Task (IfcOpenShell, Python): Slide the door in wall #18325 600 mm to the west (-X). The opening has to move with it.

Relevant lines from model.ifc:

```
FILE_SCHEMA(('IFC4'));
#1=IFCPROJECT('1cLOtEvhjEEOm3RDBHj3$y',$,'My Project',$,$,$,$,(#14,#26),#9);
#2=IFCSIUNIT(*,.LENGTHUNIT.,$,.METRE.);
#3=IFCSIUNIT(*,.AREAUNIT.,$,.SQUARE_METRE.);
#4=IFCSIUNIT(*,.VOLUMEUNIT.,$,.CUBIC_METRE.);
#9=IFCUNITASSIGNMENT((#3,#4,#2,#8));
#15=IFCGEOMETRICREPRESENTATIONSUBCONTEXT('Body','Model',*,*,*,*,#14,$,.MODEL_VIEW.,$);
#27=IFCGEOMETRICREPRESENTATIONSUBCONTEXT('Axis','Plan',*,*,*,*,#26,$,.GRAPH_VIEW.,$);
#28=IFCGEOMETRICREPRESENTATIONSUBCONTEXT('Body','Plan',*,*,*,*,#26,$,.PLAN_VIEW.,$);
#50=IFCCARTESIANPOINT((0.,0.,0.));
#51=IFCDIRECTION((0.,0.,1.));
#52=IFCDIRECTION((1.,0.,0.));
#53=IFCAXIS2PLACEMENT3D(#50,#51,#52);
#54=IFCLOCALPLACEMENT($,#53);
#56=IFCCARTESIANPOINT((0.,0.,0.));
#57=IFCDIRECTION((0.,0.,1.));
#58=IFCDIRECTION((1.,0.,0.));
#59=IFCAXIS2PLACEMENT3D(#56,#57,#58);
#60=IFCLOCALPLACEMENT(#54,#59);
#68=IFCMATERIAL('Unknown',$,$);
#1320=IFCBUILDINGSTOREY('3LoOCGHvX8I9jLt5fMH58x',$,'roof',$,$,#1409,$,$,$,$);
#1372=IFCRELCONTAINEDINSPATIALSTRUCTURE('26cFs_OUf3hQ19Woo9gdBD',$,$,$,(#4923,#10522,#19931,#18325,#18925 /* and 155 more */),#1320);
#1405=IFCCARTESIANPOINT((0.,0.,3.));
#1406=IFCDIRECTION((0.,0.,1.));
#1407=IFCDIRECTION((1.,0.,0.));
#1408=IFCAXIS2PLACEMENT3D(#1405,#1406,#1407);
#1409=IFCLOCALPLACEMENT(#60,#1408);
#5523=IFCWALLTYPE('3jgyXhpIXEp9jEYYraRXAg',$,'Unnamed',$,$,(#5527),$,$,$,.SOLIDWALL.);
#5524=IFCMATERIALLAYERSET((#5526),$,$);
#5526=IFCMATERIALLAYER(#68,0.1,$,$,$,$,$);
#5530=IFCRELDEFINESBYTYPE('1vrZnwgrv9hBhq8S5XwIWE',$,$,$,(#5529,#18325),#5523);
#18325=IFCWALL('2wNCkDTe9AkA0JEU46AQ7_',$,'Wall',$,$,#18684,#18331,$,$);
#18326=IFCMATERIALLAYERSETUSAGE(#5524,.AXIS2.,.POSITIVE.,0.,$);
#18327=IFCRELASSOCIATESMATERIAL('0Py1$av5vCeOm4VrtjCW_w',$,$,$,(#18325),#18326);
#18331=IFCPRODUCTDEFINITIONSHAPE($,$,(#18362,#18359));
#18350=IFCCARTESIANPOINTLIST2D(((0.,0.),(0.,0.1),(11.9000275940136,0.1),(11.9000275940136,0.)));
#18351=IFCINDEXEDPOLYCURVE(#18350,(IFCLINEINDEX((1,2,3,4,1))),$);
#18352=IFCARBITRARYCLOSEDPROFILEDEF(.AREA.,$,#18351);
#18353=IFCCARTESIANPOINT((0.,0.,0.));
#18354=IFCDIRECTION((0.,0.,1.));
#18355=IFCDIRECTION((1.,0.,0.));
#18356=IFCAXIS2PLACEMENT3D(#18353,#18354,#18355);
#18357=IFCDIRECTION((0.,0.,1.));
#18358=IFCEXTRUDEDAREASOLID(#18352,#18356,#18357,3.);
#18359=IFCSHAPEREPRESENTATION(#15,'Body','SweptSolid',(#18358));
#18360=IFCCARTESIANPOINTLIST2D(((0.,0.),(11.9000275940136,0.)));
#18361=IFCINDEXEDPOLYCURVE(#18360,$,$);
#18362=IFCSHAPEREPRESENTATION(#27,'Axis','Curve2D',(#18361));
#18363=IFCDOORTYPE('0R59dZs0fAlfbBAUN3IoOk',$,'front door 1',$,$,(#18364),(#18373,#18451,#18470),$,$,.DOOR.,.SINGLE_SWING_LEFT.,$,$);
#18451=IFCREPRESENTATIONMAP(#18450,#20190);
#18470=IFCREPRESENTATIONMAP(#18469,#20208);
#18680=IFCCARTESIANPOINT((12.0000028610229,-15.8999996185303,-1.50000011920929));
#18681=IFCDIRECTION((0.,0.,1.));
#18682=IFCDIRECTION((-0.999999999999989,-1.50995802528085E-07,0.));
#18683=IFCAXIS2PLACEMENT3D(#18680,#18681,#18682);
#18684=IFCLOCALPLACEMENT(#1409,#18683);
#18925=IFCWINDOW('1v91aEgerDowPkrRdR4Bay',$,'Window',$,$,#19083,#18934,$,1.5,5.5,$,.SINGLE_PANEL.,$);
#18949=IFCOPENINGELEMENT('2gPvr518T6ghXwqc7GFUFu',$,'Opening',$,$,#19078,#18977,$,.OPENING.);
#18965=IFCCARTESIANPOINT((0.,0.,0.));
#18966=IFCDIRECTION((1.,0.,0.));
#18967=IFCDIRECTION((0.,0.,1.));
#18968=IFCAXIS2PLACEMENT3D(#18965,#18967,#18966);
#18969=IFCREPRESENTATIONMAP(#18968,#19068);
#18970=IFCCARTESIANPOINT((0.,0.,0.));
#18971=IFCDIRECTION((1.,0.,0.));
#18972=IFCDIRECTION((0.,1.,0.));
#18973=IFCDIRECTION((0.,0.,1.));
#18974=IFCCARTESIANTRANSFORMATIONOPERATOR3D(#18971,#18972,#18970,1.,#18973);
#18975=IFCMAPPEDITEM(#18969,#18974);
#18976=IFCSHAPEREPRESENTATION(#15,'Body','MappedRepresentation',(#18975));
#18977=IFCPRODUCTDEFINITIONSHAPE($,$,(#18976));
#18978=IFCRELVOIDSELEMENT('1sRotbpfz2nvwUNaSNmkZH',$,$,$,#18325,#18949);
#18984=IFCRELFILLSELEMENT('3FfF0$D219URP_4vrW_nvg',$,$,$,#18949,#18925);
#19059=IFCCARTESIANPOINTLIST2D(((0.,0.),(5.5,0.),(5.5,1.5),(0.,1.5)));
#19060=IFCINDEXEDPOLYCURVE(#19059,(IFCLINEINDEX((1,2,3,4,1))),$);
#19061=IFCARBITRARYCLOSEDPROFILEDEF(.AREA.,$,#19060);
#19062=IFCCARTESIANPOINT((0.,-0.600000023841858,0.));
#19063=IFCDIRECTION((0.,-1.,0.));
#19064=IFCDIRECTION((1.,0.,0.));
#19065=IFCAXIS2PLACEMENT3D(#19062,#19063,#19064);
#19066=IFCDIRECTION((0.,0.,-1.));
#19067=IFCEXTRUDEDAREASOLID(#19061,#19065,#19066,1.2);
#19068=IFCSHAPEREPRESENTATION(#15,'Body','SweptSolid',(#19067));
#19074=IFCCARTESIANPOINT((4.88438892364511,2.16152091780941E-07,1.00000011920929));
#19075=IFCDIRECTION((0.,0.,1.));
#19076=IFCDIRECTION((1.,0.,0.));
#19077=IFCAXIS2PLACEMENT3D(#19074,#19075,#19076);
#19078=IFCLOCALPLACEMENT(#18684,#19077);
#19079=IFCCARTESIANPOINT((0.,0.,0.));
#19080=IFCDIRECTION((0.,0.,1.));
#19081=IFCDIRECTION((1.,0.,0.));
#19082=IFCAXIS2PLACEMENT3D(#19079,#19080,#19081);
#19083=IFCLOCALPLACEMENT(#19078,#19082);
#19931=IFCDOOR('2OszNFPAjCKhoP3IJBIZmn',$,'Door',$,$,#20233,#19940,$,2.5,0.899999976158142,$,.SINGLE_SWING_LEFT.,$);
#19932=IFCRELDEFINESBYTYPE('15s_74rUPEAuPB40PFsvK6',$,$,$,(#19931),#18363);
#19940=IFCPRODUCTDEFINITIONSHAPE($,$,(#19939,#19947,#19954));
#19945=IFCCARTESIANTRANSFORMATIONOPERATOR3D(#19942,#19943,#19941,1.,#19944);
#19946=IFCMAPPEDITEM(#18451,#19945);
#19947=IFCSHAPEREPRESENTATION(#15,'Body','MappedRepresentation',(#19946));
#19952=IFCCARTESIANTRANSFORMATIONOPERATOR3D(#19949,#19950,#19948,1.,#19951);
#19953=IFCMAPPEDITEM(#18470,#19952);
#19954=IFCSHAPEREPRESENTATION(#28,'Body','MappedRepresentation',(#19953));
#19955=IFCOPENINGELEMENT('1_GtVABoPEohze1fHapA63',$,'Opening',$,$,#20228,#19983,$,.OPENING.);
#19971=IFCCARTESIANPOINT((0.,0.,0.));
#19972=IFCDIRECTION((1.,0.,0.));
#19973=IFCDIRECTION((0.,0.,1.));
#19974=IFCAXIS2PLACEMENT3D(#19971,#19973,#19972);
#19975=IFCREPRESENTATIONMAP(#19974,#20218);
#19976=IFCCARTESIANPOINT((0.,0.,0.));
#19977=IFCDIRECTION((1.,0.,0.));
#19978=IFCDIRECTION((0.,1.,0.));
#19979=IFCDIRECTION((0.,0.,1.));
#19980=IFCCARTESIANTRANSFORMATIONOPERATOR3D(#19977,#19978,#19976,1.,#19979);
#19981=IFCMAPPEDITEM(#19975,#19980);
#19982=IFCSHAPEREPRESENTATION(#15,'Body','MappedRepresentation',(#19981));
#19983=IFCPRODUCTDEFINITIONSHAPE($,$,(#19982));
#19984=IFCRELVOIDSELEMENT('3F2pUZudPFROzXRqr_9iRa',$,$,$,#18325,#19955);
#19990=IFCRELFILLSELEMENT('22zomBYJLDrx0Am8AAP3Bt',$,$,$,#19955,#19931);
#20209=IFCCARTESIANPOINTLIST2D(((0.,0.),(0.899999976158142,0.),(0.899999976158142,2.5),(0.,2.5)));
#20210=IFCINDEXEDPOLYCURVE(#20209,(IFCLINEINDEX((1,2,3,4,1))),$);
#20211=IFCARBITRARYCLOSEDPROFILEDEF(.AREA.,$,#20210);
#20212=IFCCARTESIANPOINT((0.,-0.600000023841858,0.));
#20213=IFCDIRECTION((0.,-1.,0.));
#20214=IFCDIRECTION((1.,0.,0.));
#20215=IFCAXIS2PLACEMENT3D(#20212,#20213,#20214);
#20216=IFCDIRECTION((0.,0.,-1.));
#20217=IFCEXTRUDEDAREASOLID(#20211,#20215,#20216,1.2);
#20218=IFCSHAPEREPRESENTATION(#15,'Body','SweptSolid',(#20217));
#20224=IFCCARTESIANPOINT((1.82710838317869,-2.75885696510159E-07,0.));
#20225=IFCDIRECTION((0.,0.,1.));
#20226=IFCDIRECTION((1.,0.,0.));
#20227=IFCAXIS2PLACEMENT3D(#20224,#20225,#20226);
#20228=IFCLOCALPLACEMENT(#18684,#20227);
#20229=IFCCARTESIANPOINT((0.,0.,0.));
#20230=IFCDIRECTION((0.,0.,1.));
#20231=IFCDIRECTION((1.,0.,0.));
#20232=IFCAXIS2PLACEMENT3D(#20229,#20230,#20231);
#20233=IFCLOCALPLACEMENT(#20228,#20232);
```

```python
import ifcopenshell
import ifcopenshell.api.geometry
import ifcopenshell.util.placement

model = ifcopenshell.open("model.ifc")

door = model.by_guid("2OszNFPAjCKhoP3IJBIZmn")
opening = door.FillsVoids[0].RelatingOpeningElement
wall = opening.VoidsElements[0].RelatingBuildingElement

wall_matrix = ifcopenshell.util.placement.get_local_placement(wall.ObjectPlacement)
shift = wall_matrix[:3, 0] * 0.6
before = ifcopenshell.util.placement.get_local_placement(door.ObjectPlacement)[:3, 3].copy()

# The door is placed relative to its opening, so it follows when the opening moves.
matrix = ifcopenshell.util.placement.get_local_placement(opening.ObjectPlacement)
matrix[:3, 3] += shift
ifcopenshell.api.geometry.edit_object_placement(
    model, product=opening, matrix=matrix, is_si=False, should_transform_children=True
)

after = ifcopenshell.util.placement.get_local_placement(door.ObjectPlacement)[:3, 3]
print("door moved by", (after - before).round(3) + 0.0)

model.write("model_rev.ifc")
```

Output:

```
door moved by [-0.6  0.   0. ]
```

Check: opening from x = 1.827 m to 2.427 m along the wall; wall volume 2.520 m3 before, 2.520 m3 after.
